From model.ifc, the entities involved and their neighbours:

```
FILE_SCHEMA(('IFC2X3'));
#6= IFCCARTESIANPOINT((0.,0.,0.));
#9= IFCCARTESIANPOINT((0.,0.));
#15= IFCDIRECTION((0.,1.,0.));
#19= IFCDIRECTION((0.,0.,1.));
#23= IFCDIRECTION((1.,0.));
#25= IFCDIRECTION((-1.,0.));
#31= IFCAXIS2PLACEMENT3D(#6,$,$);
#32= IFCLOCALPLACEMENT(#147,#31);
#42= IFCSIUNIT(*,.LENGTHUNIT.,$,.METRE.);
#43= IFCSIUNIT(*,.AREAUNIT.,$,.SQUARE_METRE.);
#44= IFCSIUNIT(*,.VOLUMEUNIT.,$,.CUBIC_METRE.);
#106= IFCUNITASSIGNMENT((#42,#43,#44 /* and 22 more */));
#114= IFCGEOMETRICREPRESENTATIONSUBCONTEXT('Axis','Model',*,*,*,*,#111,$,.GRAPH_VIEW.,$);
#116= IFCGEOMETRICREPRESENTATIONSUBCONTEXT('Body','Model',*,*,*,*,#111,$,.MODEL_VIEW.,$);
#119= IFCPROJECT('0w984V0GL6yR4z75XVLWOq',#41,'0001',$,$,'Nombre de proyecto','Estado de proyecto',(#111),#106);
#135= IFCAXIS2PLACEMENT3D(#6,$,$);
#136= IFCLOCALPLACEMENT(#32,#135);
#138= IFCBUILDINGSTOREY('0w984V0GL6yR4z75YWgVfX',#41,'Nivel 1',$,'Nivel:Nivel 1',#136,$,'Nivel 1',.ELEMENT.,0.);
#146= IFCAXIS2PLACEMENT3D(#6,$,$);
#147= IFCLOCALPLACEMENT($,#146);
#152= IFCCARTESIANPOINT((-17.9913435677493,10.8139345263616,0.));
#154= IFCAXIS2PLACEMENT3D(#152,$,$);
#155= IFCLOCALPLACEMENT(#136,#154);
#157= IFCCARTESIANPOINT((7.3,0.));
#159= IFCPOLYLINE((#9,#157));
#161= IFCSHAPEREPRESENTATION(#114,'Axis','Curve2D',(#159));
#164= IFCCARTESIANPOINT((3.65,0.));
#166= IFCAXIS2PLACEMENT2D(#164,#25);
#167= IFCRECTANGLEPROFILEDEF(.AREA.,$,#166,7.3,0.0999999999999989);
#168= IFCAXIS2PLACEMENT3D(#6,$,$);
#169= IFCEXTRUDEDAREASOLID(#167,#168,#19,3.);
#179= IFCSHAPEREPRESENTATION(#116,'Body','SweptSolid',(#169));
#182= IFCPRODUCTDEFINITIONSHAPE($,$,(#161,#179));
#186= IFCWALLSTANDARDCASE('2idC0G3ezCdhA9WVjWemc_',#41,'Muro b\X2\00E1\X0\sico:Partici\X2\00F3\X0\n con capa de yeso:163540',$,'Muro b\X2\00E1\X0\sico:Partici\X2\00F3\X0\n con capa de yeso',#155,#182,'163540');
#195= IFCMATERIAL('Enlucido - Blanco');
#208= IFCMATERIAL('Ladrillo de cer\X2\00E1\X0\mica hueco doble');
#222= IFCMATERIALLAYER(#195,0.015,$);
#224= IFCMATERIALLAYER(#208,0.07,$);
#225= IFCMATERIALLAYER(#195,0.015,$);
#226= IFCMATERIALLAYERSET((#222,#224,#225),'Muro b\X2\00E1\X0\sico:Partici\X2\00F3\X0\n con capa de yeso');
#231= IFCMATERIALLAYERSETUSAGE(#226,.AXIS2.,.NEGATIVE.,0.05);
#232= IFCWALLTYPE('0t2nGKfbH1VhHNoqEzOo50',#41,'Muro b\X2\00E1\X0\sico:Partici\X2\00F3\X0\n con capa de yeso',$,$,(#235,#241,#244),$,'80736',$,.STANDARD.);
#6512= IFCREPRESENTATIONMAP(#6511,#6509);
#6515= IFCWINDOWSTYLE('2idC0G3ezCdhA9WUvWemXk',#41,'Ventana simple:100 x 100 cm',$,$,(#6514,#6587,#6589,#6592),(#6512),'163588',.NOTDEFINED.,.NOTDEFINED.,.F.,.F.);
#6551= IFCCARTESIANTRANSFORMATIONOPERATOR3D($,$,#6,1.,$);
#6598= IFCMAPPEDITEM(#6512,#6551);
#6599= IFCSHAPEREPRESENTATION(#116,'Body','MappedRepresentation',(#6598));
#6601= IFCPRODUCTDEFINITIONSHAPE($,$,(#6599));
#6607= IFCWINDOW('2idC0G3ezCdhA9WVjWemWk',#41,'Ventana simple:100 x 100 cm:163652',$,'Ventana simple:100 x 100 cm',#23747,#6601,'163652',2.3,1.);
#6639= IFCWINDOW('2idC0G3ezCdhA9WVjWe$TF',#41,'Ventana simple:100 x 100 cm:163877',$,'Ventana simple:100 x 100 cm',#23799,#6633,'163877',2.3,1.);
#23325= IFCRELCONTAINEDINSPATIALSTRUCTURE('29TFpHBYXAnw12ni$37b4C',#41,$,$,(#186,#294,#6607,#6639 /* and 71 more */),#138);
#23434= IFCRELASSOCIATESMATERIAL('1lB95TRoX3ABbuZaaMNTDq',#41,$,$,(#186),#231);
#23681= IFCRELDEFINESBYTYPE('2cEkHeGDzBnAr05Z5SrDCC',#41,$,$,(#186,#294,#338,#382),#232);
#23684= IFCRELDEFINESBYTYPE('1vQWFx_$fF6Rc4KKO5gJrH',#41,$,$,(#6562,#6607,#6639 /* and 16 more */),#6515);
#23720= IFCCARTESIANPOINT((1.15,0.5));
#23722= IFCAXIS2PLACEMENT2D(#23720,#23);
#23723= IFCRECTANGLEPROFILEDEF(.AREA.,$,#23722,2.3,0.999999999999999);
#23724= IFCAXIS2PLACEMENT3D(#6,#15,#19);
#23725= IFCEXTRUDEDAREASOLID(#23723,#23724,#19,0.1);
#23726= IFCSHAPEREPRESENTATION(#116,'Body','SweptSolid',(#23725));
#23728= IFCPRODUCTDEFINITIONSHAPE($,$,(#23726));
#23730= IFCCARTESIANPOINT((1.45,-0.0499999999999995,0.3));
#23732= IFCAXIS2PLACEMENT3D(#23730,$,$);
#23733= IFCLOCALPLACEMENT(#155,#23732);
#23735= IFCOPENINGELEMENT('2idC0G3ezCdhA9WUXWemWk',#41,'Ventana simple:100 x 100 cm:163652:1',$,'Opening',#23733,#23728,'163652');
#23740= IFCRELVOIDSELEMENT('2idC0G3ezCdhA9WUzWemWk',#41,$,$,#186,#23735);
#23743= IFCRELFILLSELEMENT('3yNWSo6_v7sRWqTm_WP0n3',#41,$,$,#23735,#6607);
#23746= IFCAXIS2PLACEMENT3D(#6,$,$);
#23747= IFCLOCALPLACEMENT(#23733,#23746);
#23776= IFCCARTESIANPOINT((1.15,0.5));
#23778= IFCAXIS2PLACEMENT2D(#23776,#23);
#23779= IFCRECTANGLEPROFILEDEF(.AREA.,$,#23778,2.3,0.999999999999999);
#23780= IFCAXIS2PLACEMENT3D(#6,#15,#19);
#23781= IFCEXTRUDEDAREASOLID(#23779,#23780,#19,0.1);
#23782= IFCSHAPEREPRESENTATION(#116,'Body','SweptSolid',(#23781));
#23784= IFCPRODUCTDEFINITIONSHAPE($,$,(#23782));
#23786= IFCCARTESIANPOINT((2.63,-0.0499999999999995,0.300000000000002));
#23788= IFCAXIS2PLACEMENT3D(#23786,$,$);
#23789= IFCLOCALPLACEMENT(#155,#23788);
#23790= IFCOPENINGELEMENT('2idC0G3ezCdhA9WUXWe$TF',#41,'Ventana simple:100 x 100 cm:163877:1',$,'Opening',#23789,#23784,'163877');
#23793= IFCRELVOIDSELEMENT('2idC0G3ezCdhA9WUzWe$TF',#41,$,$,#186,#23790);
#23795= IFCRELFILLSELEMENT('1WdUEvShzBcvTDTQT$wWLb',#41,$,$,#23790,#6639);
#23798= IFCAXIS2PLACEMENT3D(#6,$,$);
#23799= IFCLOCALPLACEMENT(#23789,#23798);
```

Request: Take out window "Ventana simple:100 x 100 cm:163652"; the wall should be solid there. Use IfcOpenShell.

```python
import ifcopenshell
import ifcopenshell.api.feature
import ifcopenshell.api.root
import ifcopenshell.geom
import ifcopenshell.util.shape

model = ifcopenshell.open("model.ifc")
settings = ifcopenshell.geom.settings()


def volume(element):
    """Net volume in cubic metres, openings subtracted."""
    shape = ifcopenshell.geom.create_shape(settings, element)
    return ifcopenshell.util.shape.get_volume(shape.geometry)


window = model.by_id(6607)
opening = window.FillsVoids[0].RelatingOpeningElement
wall = opening.VoidsElements[0].RelatingBuildingElement
before = volume(wall)

ifcopenshell.api.root.remove_product(model, product=window)
ifcopenshell.api.feature.remove_feature(model, feature=opening)

after = volume(wall)

print(f"wall volume {before:.3f} -> {after:.3f} m3")

model.write("model_v2.ifc")
```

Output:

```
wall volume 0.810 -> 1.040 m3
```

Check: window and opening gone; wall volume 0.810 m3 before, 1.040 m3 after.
